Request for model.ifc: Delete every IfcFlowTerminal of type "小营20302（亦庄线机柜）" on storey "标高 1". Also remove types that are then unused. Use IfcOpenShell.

First a look at what the model holds.

```python
import ifcopenshell
import ifcopenshell.util.element

model = ifcopenshell.open("model.ifc")
print(model.schema)
storey = next(s for s in model.by_type("IfcBuildingStorey") if s.Name == "标高 1")
terminals = [e for e in ifcopenshell.util.element.get_decomposition(storey) if e.is_a("IfcFlowTerminal")]
seen = {}
for e in terminals:
    element_type = ifcopenshell.util.element.get_type(e)
    name = element_type.Name if element_type not in (None, e) else None
    seen[name] = seen.get(name, 0) + 1
for name, count in sorted(seen.items(), key=str):
    print(count, "x", name)
```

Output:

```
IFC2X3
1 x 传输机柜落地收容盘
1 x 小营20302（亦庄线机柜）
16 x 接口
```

```python
import ifcopenshell
import ifcopenshell.api.root
import ifcopenshell.util.element

model = ifcopenshell.open("model.ifc")

storey = next(s for s in model.by_type("IfcBuildingStorey") if s.Name == "标高 1")
terminals = [e for e in ifcopenshell.util.element.get_decomposition(storey) if e.is_a("IfcFlowTerminal")]
targets = [e for e in terminals if (t := ifcopenshell.util.element.get_type(e)) not in (None, e) and t.Name == "小营20302（亦庄线机柜）"]
types = {ifcopenshell.util.element.get_type(e) for e in targets} - {None, *targets}

for e in targets:
    ifcopenshell.api.root.remove_product(model, product=e)
print(len(targets), "removed")

unused = [t for t in types if not ifcopenshell.util.element.get_types(t)]
for t in unused:
    ifcopenshell.api.root.remove_product(model, product=t)
print(len(unused), "unused types removed")

model.write("model-out.ifc")
```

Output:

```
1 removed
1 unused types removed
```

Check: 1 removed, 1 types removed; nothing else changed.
